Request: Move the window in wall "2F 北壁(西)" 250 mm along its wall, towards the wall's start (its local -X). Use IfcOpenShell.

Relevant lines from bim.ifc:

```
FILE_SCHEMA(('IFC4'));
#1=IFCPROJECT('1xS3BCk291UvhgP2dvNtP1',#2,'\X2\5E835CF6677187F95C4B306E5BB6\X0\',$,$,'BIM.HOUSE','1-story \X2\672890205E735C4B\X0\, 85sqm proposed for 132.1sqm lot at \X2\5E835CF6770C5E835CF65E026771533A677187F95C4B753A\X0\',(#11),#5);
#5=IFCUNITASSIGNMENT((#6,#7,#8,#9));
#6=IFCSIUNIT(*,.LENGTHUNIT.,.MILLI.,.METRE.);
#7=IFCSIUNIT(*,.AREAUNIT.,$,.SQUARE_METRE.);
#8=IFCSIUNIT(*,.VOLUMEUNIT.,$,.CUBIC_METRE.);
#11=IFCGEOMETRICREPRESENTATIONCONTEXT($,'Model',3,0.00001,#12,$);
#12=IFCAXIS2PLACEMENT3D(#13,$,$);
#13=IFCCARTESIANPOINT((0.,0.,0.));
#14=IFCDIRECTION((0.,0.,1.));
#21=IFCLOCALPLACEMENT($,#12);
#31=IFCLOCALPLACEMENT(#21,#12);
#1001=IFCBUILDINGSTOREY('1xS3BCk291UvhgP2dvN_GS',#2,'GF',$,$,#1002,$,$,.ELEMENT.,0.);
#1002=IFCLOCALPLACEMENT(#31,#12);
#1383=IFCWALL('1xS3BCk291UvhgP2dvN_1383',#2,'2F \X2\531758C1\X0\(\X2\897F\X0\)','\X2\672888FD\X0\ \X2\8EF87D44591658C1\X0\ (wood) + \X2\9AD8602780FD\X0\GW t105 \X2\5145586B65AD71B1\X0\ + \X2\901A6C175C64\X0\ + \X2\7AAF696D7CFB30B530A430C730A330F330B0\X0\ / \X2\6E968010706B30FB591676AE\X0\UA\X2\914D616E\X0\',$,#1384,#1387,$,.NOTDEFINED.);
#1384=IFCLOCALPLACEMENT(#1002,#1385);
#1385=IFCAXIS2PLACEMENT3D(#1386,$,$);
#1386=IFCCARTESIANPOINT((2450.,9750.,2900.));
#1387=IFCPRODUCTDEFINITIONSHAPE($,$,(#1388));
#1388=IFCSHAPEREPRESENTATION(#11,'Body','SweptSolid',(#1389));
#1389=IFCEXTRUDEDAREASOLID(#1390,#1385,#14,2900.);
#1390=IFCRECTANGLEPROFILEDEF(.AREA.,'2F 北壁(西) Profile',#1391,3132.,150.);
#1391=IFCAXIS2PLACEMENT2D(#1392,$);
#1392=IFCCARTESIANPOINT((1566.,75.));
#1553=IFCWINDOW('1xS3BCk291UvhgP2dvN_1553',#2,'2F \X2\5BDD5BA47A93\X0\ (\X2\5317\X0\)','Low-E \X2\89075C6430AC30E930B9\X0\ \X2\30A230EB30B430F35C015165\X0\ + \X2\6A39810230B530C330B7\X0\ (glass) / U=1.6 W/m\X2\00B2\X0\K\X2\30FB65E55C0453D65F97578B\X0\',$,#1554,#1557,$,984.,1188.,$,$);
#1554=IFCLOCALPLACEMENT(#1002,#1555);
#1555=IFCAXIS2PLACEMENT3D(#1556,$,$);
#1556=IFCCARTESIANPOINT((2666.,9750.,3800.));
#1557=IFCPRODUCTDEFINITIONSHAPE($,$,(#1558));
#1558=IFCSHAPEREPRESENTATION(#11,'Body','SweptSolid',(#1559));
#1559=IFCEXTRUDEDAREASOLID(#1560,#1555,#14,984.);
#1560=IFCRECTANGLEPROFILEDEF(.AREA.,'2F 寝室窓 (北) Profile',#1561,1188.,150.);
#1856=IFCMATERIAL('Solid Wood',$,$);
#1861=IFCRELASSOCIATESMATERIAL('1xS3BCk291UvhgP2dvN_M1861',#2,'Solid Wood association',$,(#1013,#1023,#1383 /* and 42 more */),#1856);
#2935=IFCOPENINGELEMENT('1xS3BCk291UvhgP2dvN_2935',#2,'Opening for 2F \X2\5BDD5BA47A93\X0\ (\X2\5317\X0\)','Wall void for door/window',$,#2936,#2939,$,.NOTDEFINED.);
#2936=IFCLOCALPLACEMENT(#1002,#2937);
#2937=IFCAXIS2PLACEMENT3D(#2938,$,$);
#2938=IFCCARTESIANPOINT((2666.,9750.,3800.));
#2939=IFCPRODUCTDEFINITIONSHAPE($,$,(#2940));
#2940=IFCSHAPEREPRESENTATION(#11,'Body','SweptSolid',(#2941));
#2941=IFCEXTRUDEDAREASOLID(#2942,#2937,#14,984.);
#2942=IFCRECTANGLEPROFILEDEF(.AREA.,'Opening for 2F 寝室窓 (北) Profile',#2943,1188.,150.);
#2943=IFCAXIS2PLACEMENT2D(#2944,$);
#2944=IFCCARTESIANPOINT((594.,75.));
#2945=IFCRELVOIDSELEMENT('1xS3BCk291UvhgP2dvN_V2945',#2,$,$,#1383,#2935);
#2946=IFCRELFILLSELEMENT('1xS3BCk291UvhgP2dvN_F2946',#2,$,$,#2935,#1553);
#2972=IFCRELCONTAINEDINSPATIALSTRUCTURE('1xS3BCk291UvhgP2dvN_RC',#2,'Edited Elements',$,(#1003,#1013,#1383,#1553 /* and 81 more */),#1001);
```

```python
import ifcopenshell
import ifcopenshell.api.geometry
import ifcopenshell.util.placement
import ifcopenshell.util.unit

model = ifcopenshell.open("bim.ifc")
unit_scale = ifcopenshell.util.unit.calculate_unit_scale(model)

window = model.by_id(1553)
opening = window.FillsVoids[0].RelatingOpeningElement
wall = opening.VoidsElements[0].RelatingBuildingElement

wall_matrix = ifcopenshell.util.placement.get_local_placement(wall.ObjectPlacement)
shift = wall_matrix[:3, 0] * -0.25 / unit_scale
before = ifcopenshell.util.placement.get_local_placement(window.ObjectPlacement)[:3, 3].copy()

# The window is not placed relative to its opening, so move both.
for product in (opening, window):
    matrix = ifcopenshell.util.placement.get_local_placement(product.ObjectPlacement)
    matrix[:3, 3] += shift
    ifcopenshell.api.geometry.edit_object_placement(model, product=product, matrix=matrix, is_si=False)

after = ifcopenshell.util.placement.get_local_placement(window.ObjectPlacement)[:3, 3]
print("window moved by", (after - before).round(3) + 0.0)

model.write("bim_edited.ifc")
```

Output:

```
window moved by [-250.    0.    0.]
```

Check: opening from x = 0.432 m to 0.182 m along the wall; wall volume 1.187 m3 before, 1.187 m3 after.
